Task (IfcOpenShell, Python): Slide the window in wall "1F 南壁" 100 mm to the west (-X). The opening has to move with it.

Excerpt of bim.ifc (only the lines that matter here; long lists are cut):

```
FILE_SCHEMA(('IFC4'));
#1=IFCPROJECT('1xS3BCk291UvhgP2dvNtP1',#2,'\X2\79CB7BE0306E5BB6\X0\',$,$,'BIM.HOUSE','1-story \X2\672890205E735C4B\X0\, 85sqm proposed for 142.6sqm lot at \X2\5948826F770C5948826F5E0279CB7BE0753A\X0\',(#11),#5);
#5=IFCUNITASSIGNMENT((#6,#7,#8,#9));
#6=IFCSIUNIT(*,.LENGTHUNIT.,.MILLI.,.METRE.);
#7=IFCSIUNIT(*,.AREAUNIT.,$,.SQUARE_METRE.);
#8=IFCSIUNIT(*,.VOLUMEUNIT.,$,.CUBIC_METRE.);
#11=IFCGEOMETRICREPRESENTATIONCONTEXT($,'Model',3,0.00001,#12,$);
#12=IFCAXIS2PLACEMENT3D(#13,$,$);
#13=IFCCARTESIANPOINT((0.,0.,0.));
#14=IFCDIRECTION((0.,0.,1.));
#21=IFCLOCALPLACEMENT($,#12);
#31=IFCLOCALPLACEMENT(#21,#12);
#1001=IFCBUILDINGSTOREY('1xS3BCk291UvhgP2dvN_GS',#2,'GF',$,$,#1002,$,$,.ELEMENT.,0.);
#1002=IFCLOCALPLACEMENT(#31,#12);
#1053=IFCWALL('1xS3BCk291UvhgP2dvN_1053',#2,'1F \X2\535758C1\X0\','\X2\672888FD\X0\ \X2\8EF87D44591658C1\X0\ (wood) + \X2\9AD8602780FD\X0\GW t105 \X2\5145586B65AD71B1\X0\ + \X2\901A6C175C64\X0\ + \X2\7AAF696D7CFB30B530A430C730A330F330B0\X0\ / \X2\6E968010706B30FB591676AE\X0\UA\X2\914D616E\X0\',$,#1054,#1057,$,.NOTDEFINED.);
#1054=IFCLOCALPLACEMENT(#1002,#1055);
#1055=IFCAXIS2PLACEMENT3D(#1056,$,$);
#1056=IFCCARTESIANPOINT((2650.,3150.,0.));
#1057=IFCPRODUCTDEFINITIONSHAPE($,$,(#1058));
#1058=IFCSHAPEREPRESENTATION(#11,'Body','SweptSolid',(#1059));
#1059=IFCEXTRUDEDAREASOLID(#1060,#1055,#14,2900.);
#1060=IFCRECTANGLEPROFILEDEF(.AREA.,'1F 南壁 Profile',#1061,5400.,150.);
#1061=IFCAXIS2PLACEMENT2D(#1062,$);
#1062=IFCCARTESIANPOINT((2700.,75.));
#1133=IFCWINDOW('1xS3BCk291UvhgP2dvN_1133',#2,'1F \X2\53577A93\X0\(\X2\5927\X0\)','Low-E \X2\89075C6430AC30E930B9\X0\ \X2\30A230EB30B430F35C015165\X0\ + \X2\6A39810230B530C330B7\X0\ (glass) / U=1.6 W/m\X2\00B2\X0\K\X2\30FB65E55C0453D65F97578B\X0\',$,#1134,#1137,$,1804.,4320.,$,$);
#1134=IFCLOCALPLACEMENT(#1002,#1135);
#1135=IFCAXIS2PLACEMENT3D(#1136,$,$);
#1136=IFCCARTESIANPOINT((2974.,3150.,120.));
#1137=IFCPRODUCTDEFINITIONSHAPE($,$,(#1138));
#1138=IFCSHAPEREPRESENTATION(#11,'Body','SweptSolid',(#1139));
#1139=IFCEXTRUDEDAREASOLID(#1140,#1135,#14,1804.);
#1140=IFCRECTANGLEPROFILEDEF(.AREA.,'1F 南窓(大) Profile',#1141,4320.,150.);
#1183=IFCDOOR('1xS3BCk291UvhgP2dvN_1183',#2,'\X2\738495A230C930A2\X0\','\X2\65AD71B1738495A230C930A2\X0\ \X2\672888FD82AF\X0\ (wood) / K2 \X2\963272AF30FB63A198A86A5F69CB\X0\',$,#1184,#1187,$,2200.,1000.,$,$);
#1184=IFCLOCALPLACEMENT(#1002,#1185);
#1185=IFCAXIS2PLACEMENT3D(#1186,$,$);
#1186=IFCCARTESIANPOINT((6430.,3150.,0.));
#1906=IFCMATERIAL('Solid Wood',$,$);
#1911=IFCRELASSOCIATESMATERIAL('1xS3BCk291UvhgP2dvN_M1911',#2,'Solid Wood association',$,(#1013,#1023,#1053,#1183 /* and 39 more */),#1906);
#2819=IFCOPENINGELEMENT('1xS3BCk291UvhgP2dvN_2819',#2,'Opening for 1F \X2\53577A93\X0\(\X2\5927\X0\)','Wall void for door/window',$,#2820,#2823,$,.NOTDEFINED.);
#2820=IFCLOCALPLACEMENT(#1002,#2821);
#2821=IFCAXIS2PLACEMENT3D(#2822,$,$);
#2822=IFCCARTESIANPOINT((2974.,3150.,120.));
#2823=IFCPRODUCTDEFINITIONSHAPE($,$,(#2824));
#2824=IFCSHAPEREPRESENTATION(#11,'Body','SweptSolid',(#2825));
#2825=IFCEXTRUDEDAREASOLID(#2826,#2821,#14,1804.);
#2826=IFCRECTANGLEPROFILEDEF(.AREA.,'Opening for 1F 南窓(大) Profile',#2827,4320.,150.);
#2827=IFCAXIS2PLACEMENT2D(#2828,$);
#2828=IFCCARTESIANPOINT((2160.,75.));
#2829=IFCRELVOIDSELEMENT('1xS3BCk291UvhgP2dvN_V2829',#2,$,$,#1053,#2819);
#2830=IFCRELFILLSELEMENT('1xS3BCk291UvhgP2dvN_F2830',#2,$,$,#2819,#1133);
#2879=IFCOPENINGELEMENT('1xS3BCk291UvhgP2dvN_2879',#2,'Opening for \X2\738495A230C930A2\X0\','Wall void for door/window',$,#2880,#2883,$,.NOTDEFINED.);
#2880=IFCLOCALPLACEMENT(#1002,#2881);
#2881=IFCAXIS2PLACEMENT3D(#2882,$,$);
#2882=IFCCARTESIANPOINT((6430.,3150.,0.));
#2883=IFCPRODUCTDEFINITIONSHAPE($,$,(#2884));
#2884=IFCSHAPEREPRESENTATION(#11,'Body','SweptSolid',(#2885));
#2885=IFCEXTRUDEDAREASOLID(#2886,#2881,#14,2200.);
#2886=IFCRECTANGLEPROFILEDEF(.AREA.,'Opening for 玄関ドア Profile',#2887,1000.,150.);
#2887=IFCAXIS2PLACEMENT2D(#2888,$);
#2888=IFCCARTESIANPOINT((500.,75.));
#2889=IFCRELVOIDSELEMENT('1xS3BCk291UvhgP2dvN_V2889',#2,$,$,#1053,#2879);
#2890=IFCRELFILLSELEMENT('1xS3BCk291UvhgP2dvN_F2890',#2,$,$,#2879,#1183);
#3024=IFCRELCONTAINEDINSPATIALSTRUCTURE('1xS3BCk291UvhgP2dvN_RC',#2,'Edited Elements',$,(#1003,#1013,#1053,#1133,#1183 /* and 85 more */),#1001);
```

```python
import ifcopenshell
import ifcopenshell.api.geometry
import ifcopenshell.util.placement
import ifcopenshell.util.unit

model = ifcopenshell.open("bim.ifc")
unit_scale = ifcopenshell.util.unit.calculate_unit_scale(model)

window = model.by_guid("1xS3BCk291UvhgP2dvN_1133")
opening = window.FillsVoids[0].RelatingOpeningElement
wall = opening.VoidsElements[0].RelatingBuildingElement

wall_matrix = ifcopenshell.util.placement.get_local_placement(wall.ObjectPlacement)
shift = wall_matrix[:3, 0] * -0.1 / unit_scale
before = ifcopenshell.util.placement.get_local_placement(window.ObjectPlacement)[:3, 3].copy()

# The window is not placed relative to its opening, so move both.
for product in (opening, window):
    matrix = ifcopenshell.util.placement.get_local_placement(product.ObjectPlacement)
    matrix[:3, 3] += shift
    ifcopenshell.api.geometry.edit_object_placement(model, product=product, matrix=matrix, is_si=False)

after = ifcopenshell.util.placement.get_local_placement(window.ObjectPlacement)[:3, 3]
print("window moved by", (after - before).round(3) + 0.0)

model.write("bim-out.ifc")
```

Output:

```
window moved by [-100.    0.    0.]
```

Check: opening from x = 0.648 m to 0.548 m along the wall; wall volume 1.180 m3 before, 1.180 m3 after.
